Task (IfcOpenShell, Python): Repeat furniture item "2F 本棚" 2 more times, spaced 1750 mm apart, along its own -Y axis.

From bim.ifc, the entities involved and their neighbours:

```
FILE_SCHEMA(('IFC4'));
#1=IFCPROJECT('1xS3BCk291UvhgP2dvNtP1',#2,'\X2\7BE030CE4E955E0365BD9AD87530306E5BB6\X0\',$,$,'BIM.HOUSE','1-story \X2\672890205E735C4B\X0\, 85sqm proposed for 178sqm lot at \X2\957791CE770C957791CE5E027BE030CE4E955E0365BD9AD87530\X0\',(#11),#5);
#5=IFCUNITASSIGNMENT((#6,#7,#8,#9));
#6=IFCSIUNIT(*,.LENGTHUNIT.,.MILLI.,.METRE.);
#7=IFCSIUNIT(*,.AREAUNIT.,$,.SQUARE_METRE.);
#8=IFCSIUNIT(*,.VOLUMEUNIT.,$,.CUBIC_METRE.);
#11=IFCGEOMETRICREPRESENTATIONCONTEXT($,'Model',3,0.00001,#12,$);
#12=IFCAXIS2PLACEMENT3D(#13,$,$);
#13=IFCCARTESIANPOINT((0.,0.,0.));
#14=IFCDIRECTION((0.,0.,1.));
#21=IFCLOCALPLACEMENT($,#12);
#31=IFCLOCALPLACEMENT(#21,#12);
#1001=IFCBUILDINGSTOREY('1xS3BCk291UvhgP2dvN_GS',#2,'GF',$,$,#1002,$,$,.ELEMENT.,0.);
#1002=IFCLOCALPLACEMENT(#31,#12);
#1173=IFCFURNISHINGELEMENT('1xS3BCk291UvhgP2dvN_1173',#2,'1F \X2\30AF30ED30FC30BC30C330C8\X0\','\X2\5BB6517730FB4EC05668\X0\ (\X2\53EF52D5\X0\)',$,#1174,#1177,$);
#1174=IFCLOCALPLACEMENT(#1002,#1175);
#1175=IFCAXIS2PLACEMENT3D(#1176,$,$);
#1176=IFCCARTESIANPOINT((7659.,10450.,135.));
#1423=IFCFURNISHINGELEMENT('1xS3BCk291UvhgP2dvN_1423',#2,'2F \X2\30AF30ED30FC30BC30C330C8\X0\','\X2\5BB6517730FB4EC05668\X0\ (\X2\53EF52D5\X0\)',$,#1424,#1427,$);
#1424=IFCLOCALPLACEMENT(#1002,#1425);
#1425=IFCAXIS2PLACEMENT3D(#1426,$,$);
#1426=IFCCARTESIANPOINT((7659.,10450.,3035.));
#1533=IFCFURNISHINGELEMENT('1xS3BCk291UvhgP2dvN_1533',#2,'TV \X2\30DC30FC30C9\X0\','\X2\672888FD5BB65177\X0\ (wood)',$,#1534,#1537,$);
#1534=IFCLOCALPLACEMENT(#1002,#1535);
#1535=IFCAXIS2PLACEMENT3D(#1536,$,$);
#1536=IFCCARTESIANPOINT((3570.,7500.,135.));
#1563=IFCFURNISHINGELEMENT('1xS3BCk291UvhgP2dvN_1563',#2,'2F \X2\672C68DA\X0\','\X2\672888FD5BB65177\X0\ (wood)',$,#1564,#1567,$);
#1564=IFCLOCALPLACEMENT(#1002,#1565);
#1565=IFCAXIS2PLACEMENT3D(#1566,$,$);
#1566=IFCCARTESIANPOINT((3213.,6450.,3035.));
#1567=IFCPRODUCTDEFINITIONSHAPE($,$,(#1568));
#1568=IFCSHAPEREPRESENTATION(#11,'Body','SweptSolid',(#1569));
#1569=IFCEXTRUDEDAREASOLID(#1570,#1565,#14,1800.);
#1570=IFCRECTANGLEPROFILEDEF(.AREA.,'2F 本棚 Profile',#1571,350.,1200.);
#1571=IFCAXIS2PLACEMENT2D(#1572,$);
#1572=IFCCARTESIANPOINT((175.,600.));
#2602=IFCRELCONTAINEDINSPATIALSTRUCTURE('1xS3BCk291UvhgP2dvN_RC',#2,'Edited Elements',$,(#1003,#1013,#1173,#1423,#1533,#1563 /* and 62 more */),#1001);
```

```python
import ifcopenshell
import ifcopenshell.api.geometry
import ifcopenshell.api.root
import ifcopenshell.util.element
import ifcopenshell.util.placement

model = ifcopenshell.open("bim.ifc")


def reuse_history(source, copy):
    """copy_class also copies each property set's owner history, people and application; keep the originals."""
    for rel in copy.IsDefinedBy:
        if rel.is_a("IfcRelDefinesByProperties") and (history := rel.RelatingPropertyDefinition.OwnerHistory):
            rel.RelatingPropertyDefinition.OwnerHistory = source.OwnerHistory
            ifcopenshell.util.element.remove_deep2(model, history)


source = model.by_id(1563)
base = ifcopenshell.util.placement.get_local_placement(source.ObjectPlacement)
step = -base[:3, 1] * 1750.0

for i in range(1, 3):
    copy = ifcopenshell.api.root.copy_class(model, product=source)
    copy.Representation = ifcopenshell.util.element.copy_deep(
        model, source.Representation, exclude=["IfcGeometricRepresentationContext", "IfcRepresentationMap"]
    )
    reuse_history(source, copy)
    matrix = base.copy()
    matrix[:3, 3] += i * step
    print("added at", matrix[:3, 3].round(3) + 0.0)
    ifcopenshell.api.geometry.edit_object_placement(model, product=copy, matrix=matrix, is_si=False)

model.write("bim_v2.ifc")
```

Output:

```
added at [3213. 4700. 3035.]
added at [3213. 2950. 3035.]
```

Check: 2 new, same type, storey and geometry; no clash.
